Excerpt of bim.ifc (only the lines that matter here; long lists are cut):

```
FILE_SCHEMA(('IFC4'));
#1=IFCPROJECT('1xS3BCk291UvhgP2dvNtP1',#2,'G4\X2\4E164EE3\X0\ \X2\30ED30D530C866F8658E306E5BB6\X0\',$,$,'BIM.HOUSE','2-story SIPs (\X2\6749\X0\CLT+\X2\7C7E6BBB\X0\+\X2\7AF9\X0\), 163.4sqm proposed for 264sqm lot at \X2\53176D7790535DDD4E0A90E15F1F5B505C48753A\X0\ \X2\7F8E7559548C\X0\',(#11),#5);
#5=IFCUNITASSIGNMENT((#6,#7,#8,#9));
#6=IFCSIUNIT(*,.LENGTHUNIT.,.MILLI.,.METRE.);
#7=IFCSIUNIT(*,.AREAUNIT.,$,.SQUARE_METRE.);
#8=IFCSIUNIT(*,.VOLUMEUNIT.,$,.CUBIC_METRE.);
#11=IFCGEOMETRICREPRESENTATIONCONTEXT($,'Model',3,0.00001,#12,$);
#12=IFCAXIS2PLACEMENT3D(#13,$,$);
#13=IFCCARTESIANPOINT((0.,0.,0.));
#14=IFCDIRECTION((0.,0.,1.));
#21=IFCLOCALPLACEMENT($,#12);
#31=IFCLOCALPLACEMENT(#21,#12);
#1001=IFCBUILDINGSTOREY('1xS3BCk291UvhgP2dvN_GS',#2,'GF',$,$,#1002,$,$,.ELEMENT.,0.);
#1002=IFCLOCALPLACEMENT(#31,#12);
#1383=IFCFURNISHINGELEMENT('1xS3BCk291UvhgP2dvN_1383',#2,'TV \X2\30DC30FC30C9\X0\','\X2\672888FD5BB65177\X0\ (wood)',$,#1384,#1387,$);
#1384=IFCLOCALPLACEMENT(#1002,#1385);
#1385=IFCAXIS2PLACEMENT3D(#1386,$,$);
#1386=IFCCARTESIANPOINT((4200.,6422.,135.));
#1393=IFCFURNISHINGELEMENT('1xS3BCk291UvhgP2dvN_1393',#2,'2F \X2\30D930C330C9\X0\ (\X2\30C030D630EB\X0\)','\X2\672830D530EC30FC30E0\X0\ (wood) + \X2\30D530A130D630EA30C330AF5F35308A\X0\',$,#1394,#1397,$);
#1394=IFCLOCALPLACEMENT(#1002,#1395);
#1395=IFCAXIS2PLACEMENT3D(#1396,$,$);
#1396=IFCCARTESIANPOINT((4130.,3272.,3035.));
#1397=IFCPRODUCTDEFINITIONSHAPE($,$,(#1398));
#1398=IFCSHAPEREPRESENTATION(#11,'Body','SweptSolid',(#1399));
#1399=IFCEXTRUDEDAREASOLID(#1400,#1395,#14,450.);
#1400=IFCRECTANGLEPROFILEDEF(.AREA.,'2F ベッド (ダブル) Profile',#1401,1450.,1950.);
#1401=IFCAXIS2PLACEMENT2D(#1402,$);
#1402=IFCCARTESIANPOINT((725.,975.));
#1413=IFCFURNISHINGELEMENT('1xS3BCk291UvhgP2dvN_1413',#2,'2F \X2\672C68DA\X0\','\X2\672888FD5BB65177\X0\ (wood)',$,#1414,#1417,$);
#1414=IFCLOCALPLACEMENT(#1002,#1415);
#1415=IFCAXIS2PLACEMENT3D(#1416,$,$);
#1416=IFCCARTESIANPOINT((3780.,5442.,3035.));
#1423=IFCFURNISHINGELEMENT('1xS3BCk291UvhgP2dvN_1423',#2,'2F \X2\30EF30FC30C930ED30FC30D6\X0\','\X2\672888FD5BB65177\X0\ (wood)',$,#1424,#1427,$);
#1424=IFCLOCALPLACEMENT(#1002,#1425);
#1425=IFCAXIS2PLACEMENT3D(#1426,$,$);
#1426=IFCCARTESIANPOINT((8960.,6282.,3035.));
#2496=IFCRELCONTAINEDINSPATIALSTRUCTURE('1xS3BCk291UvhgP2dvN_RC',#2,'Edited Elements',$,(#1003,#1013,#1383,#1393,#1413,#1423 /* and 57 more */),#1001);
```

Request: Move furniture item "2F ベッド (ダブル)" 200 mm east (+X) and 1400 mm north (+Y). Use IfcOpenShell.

```python
import ifcopenshell
import ifcopenshell.api.geometry
import ifcopenshell.util.placement

model = ifcopenshell.open("bim.ifc")

item = model.by_id(1393)
matrix = ifcopenshell.util.placement.get_local_placement(item.ObjectPlacement)
matrix[0, 3] += 200.0
matrix[1, 3] += 1400.0
ifcopenshell.api.geometry.edit_object_placement(model, product=item, matrix=matrix, is_si=False)

print(ifcopenshell.util.placement.get_local_placement(item.ObjectPlacement).round(3) + 0.0)

model.write("bim_updated.ifc")
```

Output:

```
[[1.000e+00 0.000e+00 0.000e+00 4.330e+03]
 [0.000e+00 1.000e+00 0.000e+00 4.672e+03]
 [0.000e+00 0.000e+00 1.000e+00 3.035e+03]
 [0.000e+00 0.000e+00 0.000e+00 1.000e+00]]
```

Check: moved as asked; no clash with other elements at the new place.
